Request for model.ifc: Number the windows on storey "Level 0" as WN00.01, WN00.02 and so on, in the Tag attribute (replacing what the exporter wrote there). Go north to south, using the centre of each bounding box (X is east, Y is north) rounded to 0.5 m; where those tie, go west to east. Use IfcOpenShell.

First a look at what the model holds.

```python
import ifcopenshell
import ifcopenshell.util.element
import ifcopenshell.util.placement

model = ifcopenshell.open("model.ifc")
print(model.schema)
storey = next(s for s in model.by_type("IfcBuildingStorey") if s.Name == "Level 0")
windows = [e for e in ifcopenshell.util.element.get_decomposition(storey) if e.is_a("IfcWindow")]
for e in sorted(windows, key=lambda e: e.id()):
    origin = ifcopenshell.util.placement.get_local_placement(e.ObjectPlacement)[:3, 3]
    print(e.id(), e.Tag, e.Name, origin.round(2) + 0.0, sep=" | ")
```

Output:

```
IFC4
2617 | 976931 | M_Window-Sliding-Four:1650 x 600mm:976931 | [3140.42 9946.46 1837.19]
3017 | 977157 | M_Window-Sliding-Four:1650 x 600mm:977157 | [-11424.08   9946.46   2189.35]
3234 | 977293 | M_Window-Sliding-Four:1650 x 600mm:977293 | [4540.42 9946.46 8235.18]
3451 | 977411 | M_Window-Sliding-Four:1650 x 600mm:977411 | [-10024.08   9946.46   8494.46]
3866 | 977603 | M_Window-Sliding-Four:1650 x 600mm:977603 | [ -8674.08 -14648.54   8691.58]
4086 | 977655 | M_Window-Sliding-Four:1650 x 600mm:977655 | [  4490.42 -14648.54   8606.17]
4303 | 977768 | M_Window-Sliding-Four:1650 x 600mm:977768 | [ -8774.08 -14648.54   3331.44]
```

```python
import ifcopenshell
import ifcopenshell.geom
import ifcopenshell.util.element
import ifcopenshell.util.shape

model = ifcopenshell.open("model.ifc")
settings = ifcopenshell.geom.settings()
settings.set("use-world-coords", True)


def centre(element):
    shape = ifcopenshell.geom.create_shape(settings, element)
    return ifcopenshell.util.shape.get_bbox_centroid(shape.geometry)


storey = next(s for s in model.by_type("IfcBuildingStorey") if s.Name == "Level 0")
windows = [e for e in ifcopenshell.util.element.get_decomposition(storey) if e.is_a("IfcWindow")]

# Insertion points can sit at a corner or the storey origin, so sort by the geometry (in metres).
centres = {e: centre(e) for e in windows}
windows.sort(key=lambda e: (-round(centres[e][1] / 0.5), centres[e][0]))

for i, e in enumerate(windows, start=1):
    number = f"WN00.{i:02d}"
    e.Tag = number
    print(e.id(), number)

model.write("model_rev.ifc")
```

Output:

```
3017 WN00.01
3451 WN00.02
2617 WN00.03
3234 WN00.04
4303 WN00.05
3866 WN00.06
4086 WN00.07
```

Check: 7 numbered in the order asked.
